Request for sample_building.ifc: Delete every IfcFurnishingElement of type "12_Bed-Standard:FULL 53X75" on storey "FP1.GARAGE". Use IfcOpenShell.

First a look at what the model holds.

```python
import ifcopenshell
import ifcopenshell.util.element

model = ifcopenshell.open("sample_building.ifc")
print(model.schema)
storey = next(s for s in model.by_type("IfcBuildingStorey") if s.Name == "FP1.GARAGE")
furniture = [e for e in ifcopenshell.util.element.get_decomposition(storey) if e.is_a("IfcFurnishingElement")]
seen = {}
for e in furniture:
    element_type = ifcopenshell.util.element.get_type(e)
    name = element_type.Name if element_type not in (None, e) else None
    seen[name] = seen.get(name, 0) + 1
for name, count in sorted(seen.items(), key=str):
    print(count, "x", name)
```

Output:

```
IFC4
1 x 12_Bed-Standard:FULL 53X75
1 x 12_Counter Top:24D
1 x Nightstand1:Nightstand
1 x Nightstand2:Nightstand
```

```python
import ifcopenshell
import ifcopenshell.api.root
import ifcopenshell.util.element

model = ifcopenshell.open("sample_building.ifc")

storey = next(s for s in model.by_type("IfcBuildingStorey") if s.Name == "FP1.GARAGE")
furniture = [e for e in ifcopenshell.util.element.get_decomposition(storey) if e.is_a("IfcFurnishingElement")]
targets = [e for e in furniture if (t := ifcopenshell.util.element.get_type(e)) not in (None, e) and t.Name == "12_Bed-Standard:FULL 53X75"]

for e in targets:
    ifcopenshell.api.root.remove_product(model, product=e)
print(len(targets), "removed")

model.write("sample_building_rev.ifc")
```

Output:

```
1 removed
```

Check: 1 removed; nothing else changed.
